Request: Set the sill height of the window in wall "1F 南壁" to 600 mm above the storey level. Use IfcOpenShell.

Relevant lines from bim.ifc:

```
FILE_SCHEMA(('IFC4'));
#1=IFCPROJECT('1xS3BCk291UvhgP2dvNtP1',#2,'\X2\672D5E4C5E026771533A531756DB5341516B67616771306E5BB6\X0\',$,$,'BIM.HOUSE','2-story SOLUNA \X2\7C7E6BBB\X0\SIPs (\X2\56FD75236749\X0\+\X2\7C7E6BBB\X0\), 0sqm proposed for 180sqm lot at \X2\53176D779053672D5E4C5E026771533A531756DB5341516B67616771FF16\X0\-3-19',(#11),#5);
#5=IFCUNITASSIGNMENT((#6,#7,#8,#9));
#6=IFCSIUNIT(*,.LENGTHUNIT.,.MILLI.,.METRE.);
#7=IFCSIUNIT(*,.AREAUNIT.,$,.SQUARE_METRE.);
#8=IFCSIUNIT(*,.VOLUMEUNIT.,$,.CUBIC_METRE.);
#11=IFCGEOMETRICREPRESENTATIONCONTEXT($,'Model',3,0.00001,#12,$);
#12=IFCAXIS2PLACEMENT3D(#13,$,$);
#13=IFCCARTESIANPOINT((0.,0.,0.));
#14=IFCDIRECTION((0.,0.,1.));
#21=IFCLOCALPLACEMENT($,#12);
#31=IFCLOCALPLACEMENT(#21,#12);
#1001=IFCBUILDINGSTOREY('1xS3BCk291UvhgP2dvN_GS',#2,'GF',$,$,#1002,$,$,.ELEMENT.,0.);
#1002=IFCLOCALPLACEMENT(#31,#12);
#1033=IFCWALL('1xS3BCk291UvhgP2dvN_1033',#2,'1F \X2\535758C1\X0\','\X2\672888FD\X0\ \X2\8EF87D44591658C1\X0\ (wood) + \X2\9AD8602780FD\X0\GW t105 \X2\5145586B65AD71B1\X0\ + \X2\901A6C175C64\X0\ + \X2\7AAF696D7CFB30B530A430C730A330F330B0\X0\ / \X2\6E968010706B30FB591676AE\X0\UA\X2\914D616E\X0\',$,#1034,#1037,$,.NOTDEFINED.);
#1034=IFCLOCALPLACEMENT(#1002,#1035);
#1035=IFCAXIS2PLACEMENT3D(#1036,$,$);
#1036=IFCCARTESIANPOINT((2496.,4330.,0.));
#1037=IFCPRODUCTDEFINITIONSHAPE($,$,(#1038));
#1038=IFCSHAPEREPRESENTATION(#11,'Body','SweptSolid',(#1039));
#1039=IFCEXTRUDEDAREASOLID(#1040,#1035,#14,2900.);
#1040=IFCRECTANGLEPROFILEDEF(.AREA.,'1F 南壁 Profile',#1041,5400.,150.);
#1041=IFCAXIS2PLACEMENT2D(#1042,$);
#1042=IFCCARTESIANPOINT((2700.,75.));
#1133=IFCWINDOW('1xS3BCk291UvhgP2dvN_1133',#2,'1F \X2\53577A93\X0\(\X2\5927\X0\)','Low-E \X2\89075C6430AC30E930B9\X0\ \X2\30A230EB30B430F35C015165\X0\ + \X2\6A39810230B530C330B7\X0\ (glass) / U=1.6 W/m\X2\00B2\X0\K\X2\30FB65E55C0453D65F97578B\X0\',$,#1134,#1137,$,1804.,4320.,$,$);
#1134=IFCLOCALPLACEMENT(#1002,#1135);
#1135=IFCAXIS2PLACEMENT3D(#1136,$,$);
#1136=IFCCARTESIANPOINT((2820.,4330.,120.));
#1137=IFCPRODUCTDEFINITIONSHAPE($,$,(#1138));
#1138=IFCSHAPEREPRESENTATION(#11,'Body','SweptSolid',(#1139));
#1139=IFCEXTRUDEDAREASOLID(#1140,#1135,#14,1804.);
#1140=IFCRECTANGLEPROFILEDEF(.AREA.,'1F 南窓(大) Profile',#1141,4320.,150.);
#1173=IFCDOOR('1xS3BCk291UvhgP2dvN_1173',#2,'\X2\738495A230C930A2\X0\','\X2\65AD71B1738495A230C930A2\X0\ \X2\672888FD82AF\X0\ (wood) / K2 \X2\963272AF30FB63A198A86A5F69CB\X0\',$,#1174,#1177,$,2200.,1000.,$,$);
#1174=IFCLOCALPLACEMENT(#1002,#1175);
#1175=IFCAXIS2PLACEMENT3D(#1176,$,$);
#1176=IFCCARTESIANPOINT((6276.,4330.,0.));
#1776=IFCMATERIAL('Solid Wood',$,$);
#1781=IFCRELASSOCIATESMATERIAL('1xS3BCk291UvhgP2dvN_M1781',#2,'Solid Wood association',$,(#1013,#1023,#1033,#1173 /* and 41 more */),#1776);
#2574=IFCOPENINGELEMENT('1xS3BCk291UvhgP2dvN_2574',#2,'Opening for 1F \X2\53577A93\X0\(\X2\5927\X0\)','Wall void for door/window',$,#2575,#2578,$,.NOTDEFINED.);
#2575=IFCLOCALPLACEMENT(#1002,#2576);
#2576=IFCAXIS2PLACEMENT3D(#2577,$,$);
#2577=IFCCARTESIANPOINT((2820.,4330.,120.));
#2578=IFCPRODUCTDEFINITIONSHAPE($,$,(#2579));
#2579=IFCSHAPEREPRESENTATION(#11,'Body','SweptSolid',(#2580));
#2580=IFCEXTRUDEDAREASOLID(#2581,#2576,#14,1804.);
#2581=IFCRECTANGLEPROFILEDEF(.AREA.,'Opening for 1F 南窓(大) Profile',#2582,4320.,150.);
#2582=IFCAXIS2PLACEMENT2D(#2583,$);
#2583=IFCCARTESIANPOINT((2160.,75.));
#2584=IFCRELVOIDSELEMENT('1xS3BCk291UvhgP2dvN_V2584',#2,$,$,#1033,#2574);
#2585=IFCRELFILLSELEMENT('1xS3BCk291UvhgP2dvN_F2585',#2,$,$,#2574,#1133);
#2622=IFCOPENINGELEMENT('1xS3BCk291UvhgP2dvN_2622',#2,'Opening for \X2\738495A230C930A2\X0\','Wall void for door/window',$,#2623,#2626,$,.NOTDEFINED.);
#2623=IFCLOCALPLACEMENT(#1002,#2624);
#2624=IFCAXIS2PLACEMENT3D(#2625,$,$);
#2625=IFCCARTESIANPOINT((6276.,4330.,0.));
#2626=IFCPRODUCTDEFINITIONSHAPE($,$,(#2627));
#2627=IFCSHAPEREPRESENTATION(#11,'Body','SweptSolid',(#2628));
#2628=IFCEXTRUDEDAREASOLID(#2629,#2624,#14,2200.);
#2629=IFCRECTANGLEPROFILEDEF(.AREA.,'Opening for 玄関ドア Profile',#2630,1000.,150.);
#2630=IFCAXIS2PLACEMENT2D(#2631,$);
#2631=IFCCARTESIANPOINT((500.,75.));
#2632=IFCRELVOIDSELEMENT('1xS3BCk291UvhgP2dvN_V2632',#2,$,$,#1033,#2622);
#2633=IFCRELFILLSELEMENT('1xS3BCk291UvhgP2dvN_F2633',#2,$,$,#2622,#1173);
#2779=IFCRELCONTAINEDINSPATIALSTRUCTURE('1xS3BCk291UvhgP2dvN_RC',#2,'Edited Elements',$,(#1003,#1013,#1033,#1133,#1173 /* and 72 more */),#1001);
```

```python
import numpy as np
import ifcopenshell
import ifcopenshell.api.geometry
import ifcopenshell.geom
import ifcopenshell.util.element
import ifcopenshell.util.placement
import ifcopenshell.util.shape
import ifcopenshell.util.unit

model = ifcopenshell.open("bim.ifc")
unit_scale = ifcopenshell.util.unit.calculate_unit_scale(model)

window = model.by_guid("1xS3BCk291UvhgP2dvN_1133")
opening = window.FillsVoids[0].RelatingOpeningElement
storey = ifcopenshell.util.element.get_container(window, ifc_class="IfcBuildingStorey")
level = ifcopenshell.util.placement.get_local_placement(storey.ObjectPlacement)[2, 3]

# The opening's origin need not be at the sill, so measure its lowest point.
shape = ifcopenshell.geom.create_shape(ifcopenshell.geom.settings(), opening)
bottom = ifcopenshell.util.shape.get_shape_bottom_elevation(shape, shape.geometry) / unit_scale
dz = level + 0.6 / unit_scale - bottom

shift = np.array([0.0, 0.0, dz])
# The window is not placed relative to its opening, so move both.
for product in (opening, window):
    matrix = ifcopenshell.util.placement.get_local_placement(product.ObjectPlacement)
    matrix[:3, 3] += shift
    ifcopenshell.api.geometry.edit_object_placement(model, product=product, matrix=matrix, is_si=False)

print(f"moved by {dz * unit_scale:+.3f} m")

model.write("bim_rev.ifc")
```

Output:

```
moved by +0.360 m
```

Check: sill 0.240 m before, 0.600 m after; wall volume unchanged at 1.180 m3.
